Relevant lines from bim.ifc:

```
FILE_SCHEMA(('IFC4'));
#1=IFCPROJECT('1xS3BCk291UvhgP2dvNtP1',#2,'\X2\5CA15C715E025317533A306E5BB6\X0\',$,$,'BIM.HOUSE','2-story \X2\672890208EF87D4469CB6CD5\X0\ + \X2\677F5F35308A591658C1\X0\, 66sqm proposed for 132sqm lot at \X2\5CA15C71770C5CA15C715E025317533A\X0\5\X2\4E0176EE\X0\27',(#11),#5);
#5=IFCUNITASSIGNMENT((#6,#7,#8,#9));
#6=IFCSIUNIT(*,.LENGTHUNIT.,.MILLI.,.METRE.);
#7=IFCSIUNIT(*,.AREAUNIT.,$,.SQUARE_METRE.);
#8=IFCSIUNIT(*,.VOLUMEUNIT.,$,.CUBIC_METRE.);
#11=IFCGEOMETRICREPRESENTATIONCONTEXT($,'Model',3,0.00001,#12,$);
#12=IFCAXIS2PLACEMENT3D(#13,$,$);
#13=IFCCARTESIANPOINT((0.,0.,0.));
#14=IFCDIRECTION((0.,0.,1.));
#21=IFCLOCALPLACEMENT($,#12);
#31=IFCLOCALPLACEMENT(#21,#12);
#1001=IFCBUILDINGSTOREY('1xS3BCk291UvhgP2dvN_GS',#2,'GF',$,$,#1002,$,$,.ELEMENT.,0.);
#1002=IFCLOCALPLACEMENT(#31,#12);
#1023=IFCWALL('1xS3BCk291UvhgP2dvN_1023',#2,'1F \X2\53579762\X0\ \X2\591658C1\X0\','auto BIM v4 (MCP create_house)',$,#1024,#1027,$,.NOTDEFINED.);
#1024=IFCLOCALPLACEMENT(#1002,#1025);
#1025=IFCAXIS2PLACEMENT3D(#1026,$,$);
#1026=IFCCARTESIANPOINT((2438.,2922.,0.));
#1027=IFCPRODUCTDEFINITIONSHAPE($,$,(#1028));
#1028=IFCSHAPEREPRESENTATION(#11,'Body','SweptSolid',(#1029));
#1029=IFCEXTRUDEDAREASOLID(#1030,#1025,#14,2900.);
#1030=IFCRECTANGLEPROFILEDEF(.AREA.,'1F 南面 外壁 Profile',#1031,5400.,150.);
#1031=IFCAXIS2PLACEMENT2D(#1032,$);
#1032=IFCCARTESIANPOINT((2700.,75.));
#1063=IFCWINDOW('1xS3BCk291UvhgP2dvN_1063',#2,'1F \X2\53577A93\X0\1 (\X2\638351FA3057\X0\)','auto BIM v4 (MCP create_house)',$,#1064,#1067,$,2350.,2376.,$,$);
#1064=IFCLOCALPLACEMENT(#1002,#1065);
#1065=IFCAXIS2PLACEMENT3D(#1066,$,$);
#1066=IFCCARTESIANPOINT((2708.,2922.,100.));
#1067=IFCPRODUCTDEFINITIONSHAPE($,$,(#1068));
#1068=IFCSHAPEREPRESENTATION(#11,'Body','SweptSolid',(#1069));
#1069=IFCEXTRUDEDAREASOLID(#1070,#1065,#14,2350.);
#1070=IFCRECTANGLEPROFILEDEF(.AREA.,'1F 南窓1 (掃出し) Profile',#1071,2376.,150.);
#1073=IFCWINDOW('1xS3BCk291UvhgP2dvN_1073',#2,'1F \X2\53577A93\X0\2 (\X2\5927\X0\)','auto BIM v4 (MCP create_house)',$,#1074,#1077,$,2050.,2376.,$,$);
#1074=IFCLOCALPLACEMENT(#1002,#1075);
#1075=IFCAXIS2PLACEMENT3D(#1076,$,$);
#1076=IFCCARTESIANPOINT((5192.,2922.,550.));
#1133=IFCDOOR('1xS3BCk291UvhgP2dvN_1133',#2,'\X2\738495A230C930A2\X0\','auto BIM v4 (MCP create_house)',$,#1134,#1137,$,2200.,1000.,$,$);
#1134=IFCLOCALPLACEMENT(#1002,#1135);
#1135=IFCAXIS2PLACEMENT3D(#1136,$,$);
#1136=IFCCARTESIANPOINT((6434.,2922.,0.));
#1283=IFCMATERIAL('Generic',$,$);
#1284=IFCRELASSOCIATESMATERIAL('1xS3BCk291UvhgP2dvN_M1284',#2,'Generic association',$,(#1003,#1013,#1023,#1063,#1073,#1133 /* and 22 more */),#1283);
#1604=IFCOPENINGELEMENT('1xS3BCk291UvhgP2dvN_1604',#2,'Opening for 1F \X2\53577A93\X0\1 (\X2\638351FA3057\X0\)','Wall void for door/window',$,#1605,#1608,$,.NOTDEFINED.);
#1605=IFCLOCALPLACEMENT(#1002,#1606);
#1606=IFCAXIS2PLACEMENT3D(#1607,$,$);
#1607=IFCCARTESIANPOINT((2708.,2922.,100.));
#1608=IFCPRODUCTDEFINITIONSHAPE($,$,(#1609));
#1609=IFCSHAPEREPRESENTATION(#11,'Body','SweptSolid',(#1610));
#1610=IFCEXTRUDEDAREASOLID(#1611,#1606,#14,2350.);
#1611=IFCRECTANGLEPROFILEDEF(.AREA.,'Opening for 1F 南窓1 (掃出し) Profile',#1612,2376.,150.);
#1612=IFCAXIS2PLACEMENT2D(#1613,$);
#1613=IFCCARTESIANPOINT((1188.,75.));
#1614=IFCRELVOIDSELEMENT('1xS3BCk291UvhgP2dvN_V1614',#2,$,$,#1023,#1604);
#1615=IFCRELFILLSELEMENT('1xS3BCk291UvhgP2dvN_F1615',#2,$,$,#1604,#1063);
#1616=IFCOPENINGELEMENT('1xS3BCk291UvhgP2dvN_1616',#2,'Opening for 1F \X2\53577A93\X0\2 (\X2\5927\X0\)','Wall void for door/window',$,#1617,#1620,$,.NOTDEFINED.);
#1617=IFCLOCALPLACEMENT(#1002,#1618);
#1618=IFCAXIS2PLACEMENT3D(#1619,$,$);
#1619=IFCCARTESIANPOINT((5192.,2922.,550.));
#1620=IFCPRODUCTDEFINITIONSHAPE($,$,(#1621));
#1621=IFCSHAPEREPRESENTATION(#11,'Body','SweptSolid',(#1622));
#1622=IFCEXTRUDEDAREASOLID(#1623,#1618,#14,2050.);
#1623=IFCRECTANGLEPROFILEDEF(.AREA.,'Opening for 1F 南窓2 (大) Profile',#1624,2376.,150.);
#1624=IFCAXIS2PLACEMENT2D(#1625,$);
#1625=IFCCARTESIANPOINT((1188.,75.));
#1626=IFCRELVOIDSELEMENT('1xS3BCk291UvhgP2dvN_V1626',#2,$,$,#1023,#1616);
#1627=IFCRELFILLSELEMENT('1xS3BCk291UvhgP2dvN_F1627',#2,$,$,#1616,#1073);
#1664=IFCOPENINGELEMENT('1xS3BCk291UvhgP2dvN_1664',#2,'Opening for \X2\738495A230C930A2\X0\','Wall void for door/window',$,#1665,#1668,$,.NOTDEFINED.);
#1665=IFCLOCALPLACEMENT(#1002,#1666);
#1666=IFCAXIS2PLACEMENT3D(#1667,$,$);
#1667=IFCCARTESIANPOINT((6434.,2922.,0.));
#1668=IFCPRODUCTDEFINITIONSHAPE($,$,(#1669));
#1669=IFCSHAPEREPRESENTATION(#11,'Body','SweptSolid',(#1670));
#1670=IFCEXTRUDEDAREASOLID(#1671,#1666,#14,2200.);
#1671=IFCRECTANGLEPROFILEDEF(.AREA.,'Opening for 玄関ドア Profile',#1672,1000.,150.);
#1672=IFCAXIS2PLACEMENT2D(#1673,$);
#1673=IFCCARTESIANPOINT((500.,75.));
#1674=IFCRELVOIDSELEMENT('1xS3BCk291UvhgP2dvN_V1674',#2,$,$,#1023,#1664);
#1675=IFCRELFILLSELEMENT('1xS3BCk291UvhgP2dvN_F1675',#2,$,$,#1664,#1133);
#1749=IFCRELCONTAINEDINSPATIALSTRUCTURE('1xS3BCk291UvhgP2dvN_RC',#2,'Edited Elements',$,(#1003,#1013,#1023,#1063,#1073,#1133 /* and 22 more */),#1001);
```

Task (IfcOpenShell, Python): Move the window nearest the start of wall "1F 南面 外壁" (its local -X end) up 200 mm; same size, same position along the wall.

```python
import numpy as np
import ifcopenshell
import ifcopenshell.api.geometry
import ifcopenshell.util.placement
import ifcopenshell.util.unit

model = ifcopenshell.open("bim.ifc")
unit_scale = ifcopenshell.util.unit.calculate_unit_scale(model)

window = model.by_guid("1xS3BCk291UvhgP2dvN_1063")
opening = window.FillsVoids[0].RelatingOpeningElement
dz = 0.2 / unit_scale

shift = np.array([0.0, 0.0, dz])
# The window is not placed relative to its opening, so move both.
for product in (opening, window):
    matrix = ifcopenshell.util.placement.get_local_placement(product.ObjectPlacement)
    matrix[:3, 3] += shift
    ifcopenshell.api.geometry.edit_object_placement(model, product=product, matrix=matrix, is_si=False)

print(f"moved by {dz * unit_scale:+.3f} m")

model.write("bim-out.ifc")
```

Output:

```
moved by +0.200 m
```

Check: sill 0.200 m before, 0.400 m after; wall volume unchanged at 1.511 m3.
